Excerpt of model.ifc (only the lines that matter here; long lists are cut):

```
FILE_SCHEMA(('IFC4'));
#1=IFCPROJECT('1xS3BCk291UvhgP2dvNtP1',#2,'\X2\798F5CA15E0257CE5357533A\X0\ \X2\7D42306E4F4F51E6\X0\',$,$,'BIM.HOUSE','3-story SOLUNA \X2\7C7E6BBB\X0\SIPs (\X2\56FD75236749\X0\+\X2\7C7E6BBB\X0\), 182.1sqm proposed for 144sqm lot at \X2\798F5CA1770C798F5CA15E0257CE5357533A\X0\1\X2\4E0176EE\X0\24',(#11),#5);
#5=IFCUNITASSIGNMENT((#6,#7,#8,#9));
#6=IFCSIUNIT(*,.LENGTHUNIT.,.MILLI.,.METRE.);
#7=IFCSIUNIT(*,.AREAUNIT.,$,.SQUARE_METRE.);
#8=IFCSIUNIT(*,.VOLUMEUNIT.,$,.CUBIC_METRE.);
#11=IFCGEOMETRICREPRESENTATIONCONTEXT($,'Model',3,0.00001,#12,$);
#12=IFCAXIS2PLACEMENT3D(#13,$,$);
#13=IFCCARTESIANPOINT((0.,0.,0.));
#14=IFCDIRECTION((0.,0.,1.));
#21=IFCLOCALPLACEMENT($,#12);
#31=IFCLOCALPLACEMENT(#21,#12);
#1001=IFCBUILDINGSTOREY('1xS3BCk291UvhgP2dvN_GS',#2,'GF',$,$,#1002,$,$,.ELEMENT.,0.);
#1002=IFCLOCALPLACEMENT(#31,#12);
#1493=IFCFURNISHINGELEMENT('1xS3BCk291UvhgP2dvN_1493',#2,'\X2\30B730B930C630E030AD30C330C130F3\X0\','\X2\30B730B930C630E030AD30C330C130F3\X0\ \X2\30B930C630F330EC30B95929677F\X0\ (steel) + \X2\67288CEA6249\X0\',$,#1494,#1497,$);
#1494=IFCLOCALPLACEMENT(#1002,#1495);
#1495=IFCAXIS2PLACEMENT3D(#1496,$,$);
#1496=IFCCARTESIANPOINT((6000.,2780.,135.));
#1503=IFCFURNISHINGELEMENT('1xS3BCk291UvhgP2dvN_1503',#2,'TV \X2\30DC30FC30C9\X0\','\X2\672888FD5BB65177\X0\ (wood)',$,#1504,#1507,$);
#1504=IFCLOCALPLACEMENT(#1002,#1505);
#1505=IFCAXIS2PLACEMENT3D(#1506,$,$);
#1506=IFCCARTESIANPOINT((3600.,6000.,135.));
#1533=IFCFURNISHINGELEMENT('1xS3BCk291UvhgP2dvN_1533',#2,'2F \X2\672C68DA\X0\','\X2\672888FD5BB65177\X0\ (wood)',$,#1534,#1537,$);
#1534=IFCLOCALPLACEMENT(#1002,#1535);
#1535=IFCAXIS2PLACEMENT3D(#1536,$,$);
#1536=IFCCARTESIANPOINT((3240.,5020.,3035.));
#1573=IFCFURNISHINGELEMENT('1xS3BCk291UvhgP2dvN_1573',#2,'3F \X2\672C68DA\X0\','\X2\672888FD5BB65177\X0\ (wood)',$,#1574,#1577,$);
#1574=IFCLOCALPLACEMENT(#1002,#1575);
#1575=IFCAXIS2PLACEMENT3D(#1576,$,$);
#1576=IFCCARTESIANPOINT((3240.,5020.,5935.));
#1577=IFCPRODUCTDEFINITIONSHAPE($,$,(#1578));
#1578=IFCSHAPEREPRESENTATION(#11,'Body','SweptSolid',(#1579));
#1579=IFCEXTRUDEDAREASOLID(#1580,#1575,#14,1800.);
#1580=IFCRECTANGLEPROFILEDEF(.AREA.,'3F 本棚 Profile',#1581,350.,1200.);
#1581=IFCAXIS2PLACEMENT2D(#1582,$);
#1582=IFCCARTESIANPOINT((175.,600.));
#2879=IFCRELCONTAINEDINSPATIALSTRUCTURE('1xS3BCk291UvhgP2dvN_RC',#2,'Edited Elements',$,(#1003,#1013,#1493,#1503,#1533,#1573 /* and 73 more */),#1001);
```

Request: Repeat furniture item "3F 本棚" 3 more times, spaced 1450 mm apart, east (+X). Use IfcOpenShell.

```python
import numpy as np
import ifcopenshell
import ifcopenshell.api.geometry
import ifcopenshell.api.root
import ifcopenshell.util.element
import ifcopenshell.util.placement
import ifcopenshell.util.unit

model = ifcopenshell.open("model.ifc")
unit_scale = ifcopenshell.util.unit.calculate_unit_scale(model)


def reuse_history(source, copy):
    """copy_class also copies each property set's owner history, people and application; keep the originals."""
    for rel in copy.IsDefinedBy:
        if rel.is_a("IfcRelDefinesByProperties") and (history := rel.RelatingPropertyDefinition.OwnerHistory):
            rel.RelatingPropertyDefinition.OwnerHistory = source.OwnerHistory
            ifcopenshell.util.element.remove_deep2(model, history)


source = model.by_guid("1xS3BCk291UvhgP2dvN_1573")
base = ifcopenshell.util.placement.get_local_placement(source.ObjectPlacement)
step = np.array([1.0, 0.0, 0.0]) * 1.45 / unit_scale

for i in range(1, 4):
    copy = ifcopenshell.api.root.copy_class(model, product=source)
    copy.Representation = ifcopenshell.util.element.copy_deep(
        model, source.Representation, exclude=["IfcGeometricRepresentationContext", "IfcRepresentationMap"]
    )
    reuse_history(source, copy)
    matrix = base.copy()
    matrix[:3, 3] += i * step
    print("added at", matrix[:3, 3].round(3) + 0.0)
    ifcopenshell.api.geometry.edit_object_placement(model, product=copy, matrix=matrix, is_si=False)

model.write("model_v2.ifc")
```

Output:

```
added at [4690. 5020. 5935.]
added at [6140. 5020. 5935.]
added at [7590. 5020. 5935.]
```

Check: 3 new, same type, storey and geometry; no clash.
